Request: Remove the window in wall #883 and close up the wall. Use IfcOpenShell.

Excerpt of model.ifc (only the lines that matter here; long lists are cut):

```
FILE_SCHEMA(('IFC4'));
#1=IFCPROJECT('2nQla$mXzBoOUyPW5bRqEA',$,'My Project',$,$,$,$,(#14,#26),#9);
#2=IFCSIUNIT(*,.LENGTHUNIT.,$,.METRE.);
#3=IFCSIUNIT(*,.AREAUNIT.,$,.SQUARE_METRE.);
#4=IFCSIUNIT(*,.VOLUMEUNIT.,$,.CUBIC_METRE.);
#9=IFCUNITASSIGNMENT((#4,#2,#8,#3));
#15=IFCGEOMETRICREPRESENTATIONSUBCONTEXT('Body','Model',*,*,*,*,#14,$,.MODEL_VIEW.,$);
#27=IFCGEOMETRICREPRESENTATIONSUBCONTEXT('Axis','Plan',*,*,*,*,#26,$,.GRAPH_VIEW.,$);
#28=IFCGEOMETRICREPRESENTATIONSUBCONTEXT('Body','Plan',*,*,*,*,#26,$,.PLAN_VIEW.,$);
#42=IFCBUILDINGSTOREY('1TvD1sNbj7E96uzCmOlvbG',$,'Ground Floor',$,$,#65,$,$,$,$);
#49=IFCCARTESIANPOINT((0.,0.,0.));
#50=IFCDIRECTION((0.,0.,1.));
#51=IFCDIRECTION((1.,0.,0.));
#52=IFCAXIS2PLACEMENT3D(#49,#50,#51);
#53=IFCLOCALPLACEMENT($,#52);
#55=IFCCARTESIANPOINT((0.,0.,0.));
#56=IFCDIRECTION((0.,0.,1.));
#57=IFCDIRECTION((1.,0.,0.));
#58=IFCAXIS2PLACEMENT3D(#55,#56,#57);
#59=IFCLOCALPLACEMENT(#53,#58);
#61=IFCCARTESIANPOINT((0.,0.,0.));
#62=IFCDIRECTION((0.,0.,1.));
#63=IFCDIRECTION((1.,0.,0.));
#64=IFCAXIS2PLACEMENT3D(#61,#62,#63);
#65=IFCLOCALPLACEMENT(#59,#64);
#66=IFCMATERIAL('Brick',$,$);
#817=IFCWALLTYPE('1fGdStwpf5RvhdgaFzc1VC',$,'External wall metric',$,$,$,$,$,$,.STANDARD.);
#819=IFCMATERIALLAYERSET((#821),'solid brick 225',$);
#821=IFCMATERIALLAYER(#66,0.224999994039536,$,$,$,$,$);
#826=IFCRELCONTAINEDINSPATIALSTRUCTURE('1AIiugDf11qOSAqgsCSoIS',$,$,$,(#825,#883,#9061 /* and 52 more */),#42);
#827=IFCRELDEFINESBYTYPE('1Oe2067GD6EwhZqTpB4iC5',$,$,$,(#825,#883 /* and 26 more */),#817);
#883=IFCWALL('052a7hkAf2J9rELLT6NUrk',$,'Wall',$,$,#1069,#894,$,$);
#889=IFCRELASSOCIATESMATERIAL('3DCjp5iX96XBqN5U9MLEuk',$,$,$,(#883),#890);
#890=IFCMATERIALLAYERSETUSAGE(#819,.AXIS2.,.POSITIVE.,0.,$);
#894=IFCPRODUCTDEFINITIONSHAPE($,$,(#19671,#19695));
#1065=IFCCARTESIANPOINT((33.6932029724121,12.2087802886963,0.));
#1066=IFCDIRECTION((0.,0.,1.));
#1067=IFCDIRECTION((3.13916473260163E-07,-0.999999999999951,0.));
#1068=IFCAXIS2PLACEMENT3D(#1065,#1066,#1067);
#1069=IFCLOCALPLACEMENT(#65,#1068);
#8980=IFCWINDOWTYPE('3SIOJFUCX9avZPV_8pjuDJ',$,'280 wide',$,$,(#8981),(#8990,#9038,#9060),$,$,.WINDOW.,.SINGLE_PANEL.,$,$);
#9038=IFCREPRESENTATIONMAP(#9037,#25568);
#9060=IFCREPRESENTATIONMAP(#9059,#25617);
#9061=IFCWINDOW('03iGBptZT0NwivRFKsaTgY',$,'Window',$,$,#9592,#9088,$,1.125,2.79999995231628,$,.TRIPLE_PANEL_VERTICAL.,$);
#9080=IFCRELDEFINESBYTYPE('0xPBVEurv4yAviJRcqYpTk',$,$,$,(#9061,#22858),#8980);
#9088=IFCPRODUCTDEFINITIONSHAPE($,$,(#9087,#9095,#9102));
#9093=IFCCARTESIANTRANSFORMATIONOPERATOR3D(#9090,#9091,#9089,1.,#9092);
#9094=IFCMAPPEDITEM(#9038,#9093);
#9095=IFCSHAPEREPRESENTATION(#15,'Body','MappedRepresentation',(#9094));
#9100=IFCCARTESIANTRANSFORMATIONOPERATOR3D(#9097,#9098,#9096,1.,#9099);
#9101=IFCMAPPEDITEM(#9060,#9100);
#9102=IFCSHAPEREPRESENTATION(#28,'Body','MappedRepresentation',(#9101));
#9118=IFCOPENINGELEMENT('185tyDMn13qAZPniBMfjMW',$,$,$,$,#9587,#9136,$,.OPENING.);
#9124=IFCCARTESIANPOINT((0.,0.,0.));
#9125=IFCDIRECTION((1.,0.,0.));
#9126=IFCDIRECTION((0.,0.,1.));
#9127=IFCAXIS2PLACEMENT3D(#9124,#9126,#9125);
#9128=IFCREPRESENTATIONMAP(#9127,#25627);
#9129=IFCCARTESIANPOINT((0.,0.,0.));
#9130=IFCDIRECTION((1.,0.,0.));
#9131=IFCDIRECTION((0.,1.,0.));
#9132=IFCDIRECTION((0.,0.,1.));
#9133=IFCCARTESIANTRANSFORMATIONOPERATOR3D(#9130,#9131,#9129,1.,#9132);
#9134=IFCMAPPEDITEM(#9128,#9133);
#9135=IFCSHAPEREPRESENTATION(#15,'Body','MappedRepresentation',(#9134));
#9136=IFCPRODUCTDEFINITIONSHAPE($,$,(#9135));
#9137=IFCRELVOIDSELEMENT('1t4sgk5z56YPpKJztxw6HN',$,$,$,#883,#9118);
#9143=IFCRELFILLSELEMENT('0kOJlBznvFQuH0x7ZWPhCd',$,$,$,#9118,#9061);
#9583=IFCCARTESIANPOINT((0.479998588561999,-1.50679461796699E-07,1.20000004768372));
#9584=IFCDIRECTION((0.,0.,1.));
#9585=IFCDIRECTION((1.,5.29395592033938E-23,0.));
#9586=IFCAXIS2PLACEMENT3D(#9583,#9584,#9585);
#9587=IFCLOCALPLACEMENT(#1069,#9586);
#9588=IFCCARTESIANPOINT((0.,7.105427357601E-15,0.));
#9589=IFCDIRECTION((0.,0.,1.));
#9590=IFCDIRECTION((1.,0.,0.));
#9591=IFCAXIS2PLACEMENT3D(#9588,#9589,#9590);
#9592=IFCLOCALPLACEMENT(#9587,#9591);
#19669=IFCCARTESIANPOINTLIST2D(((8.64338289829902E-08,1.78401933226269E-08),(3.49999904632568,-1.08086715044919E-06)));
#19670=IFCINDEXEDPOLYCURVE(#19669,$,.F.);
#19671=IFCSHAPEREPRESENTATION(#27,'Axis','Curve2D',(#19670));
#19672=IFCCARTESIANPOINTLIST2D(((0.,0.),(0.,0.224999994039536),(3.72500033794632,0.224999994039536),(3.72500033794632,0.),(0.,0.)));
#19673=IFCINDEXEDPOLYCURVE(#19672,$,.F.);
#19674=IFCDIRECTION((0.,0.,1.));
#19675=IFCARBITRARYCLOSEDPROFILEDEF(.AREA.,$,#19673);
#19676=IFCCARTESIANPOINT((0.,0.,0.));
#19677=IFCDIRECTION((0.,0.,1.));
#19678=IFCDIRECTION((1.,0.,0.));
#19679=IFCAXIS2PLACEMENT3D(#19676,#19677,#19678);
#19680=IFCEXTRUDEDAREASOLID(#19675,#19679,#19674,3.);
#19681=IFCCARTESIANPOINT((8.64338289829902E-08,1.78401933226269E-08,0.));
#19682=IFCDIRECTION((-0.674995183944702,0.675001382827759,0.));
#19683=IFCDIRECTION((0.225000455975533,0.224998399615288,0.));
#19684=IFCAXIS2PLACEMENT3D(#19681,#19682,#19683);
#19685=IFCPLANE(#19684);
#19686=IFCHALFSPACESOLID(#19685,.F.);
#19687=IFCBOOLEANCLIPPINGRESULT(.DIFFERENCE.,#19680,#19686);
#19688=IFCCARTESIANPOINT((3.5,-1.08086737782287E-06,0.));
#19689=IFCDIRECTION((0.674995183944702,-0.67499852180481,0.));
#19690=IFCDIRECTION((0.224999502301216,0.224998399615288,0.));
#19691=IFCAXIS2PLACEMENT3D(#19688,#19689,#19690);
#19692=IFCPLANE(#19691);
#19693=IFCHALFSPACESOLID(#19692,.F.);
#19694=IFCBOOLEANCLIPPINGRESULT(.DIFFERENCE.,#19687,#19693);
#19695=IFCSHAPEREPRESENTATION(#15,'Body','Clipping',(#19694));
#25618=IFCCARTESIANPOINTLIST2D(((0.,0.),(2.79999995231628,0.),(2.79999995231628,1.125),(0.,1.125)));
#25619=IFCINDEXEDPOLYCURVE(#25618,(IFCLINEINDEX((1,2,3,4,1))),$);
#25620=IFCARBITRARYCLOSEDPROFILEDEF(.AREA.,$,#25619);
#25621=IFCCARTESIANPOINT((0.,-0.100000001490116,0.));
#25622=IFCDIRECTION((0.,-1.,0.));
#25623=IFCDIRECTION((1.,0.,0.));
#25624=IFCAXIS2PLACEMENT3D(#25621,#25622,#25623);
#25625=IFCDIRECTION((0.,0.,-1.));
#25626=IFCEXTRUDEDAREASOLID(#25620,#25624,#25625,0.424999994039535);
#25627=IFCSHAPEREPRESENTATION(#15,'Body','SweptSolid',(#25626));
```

```python
import ifcopenshell
import ifcopenshell.api.feature
import ifcopenshell.api.root
import ifcopenshell.geom
import ifcopenshell.util.shape

model = ifcopenshell.open("model.ifc")
settings = ifcopenshell.geom.settings()


def volume(element):
    """Net volume in cubic metres, openings subtracted."""
    shape = ifcopenshell.geom.create_shape(settings, element)
    return ifcopenshell.util.shape.get_volume(shape.geometry)


window = model.by_guid("03iGBptZT0NwivRFKsaTgY")
opening = window.FillsVoids[0].RelatingOpeningElement
wall = opening.VoidsElements[0].RelatingBuildingElement
before = volume(wall)

ifcopenshell.api.root.remove_product(model, product=window)
ifcopenshell.api.feature.remove_feature(model, feature=opening)

after = volume(wall)

print(f"wall volume {before:.3f} -> {after:.3f} m3")

model.write("model_updated.ifc")
```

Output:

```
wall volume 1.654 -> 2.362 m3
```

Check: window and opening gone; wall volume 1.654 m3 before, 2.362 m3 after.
